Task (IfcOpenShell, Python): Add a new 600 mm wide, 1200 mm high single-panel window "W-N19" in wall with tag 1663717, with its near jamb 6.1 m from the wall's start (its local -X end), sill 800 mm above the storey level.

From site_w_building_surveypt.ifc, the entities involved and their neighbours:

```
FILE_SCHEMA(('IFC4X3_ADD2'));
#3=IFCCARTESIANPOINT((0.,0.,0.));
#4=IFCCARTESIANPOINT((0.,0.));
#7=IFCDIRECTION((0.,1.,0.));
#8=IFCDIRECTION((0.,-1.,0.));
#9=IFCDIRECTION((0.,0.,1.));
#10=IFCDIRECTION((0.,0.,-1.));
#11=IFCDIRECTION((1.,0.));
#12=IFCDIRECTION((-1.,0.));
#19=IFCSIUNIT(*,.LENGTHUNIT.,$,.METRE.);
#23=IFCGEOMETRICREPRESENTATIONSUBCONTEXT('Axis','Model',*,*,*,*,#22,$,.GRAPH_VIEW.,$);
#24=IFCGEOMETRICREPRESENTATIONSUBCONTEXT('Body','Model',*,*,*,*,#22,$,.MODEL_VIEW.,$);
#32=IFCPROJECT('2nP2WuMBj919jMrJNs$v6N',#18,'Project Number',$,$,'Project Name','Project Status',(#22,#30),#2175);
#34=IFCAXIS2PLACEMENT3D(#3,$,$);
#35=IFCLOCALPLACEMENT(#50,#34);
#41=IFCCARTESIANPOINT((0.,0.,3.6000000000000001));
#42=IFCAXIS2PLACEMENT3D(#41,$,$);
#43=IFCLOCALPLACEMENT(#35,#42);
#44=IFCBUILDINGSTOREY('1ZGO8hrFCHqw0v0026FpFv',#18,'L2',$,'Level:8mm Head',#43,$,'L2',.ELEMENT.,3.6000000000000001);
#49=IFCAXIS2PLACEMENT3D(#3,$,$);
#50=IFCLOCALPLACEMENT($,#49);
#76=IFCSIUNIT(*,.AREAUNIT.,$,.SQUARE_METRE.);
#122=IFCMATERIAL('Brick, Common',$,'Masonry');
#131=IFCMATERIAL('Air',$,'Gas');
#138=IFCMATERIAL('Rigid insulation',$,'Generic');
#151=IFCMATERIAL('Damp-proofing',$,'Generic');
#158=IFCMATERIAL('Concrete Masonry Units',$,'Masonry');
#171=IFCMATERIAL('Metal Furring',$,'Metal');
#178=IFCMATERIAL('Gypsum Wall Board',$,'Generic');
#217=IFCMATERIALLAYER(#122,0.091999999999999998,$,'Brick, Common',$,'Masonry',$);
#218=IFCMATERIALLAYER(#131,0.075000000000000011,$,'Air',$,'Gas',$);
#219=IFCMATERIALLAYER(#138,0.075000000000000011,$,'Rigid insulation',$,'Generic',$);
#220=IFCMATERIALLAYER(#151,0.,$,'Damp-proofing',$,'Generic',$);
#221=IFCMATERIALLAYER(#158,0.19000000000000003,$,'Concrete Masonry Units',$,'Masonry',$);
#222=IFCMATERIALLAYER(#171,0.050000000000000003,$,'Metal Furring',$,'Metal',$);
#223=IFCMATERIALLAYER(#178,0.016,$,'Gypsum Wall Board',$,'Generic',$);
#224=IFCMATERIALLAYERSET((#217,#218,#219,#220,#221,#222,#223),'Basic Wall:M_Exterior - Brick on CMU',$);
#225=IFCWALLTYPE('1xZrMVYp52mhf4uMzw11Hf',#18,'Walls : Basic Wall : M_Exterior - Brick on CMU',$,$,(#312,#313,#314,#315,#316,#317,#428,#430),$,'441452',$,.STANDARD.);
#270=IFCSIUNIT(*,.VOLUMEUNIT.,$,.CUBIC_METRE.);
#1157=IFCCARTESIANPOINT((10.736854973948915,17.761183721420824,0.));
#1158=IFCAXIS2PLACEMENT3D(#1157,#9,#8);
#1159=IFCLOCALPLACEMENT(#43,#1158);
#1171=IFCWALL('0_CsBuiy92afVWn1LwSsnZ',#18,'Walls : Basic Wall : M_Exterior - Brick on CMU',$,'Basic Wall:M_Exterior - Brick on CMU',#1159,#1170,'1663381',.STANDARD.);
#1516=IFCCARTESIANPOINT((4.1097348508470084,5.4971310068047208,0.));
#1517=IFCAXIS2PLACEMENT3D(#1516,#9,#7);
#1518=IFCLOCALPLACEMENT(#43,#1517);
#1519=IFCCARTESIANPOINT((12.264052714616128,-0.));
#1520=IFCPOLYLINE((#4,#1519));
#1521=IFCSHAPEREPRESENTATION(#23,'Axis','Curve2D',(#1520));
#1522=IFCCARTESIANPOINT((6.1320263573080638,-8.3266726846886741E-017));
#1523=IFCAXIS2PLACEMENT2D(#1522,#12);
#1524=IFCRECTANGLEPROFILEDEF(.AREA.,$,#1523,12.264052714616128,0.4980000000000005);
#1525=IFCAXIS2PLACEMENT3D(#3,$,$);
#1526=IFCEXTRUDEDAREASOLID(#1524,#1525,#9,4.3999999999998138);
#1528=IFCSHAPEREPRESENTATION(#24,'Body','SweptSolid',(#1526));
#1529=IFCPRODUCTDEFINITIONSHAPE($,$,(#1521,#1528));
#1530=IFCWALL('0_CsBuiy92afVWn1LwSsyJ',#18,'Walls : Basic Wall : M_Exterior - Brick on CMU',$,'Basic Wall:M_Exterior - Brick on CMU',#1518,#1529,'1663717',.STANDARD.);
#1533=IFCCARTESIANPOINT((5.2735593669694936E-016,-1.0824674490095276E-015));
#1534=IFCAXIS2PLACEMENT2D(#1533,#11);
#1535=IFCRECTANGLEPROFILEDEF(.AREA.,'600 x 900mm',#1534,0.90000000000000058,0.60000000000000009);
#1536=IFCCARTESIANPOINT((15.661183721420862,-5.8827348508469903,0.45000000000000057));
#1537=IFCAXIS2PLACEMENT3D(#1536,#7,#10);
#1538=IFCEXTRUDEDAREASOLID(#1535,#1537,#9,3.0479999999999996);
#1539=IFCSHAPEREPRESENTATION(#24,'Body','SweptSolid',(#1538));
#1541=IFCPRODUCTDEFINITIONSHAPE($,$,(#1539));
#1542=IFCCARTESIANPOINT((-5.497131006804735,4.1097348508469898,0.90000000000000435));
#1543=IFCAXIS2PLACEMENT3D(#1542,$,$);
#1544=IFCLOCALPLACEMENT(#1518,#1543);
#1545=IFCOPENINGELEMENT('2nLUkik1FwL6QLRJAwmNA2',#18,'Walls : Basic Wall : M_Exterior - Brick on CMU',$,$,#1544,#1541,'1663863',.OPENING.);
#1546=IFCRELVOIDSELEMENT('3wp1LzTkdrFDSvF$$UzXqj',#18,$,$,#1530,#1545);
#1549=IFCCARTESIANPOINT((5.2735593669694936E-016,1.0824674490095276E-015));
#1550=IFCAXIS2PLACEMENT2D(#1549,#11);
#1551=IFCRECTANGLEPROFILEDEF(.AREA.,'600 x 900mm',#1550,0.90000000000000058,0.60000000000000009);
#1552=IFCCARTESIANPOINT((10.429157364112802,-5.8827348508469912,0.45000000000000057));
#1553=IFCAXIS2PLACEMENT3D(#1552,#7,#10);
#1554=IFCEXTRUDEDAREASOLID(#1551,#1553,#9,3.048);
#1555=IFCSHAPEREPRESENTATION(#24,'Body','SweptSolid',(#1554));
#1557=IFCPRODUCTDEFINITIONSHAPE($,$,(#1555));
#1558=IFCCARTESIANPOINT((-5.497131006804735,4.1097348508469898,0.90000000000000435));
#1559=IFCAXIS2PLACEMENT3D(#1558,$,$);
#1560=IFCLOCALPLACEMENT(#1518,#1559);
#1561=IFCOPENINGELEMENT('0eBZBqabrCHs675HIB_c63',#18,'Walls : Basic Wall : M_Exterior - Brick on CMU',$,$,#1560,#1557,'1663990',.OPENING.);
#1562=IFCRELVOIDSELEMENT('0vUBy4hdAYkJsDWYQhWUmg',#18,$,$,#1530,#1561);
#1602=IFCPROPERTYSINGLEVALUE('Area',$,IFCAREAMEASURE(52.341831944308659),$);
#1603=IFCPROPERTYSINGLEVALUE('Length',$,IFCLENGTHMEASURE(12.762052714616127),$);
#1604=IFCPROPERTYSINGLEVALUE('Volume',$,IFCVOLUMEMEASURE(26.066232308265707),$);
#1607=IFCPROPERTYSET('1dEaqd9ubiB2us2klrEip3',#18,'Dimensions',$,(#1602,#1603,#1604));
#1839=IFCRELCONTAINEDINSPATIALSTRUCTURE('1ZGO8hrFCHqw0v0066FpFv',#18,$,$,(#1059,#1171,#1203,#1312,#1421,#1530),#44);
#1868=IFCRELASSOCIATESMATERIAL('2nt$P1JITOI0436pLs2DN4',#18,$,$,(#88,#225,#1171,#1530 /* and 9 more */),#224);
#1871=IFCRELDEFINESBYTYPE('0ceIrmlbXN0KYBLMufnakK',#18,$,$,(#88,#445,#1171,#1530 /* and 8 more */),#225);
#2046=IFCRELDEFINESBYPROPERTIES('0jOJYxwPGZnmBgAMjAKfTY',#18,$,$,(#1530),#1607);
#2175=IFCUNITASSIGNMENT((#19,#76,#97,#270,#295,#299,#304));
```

```python
import numpy as np
import ifcopenshell
import ifcopenshell.api.feature
import ifcopenshell.api.geometry
import ifcopenshell.api.pset
import ifcopenshell.api.root
import ifcopenshell.api.spatial
import ifcopenshell.geom
import ifcopenshell.util.element
import ifcopenshell.util.placement
import ifcopenshell.util.representation
import ifcopenshell.util.shape
import ifcopenshell.util.unit

model = ifcopenshell.open("site_w_building_surveypt.ifc")
unit_scale = ifcopenshell.util.unit.calculate_unit_scale(model)
area_scale = ifcopenshell.util.unit.calculate_unit_scale(model, "AREAUNIT")
volume_scale = ifcopenshell.util.unit.calculate_unit_scale(model, "VOLUMEUNIT")
settings = ifcopenshell.geom.settings()


def volume(element):
    """Net volume in cubic metres, openings subtracted."""
    shape = ifcopenshell.geom.create_shape(settings, element)
    return ifcopenshell.util.shape.get_volume(shape.geometry)


wall = model.by_id(1530)
storey = ifcopenshell.util.element.get_container(wall, ifc_class="IfcBuildingStorey")
context = ifcopenshell.util.representation.get_context(model, "Model", "Body", "MODEL_VIEW")
before = volume(wall)

width, height, from_end, sill = 0.6, 1.2, 6.1, 0.8  # metres

# The wall runs along its own X axis, and the end named is its -X end.
wall_shape = ifcopenshell.geom.create_shape(settings, wall)
x, y, z = ifcopenshell.util.shape.get_vertices(wall_shape.geometry).T
start = x.min() + from_end
face, thickness = float(y.min()), float(y.max() - y.min())
wall_matrix = ifcopenshell.util.placement.get_local_placement(wall.ObjectPlacement)
level = ifcopenshell.util.placement.get_local_placement(storey.ObjectPlacement)[2, 3]


def in_wall(x, y):
    """Placement at x, y metres in the wall's axes, at sill height."""
    matrix = wall_matrix.copy()
    matrix[:, 3] = wall_matrix @ np.array([x / unit_scale, y / unit_scale, 0.0, 1.0])
    matrix[2, 3] = level + sill / unit_scale
    return matrix


# Opening: a box that overshoots both wall faces by 50 mm.
opening = ifcopenshell.api.root.create_entity(model, ifc_class="IfcOpeningElement", predefined_type="OPENING")
box = ifcopenshell.api.geometry.add_wall_representation(
    model, context=context, length=width, height=height, thickness=thickness + 0.1
)
ifcopenshell.api.geometry.assign_representation(model, product=opening, representation=box)
ifcopenshell.api.geometry.edit_object_placement(model, product=opening, matrix=in_wall(start, face - 0.05), is_si=False)
ifcopenshell.api.feature.add_feature(model, feature=opening, element=wall)

window = ifcopenshell.api.root.create_entity(model, ifc_class="IfcWindow", name="W-N19", predefined_type="WINDOW")
window.OverallWidth, window.OverallHeight = width / unit_scale, height / unit_scale
window.PartitioningType = "SINGLE_PANEL"
body = ifcopenshell.api.geometry.add_window_representation(
    model,
    context=context,
    overall_width=window.OverallWidth,
    overall_height=window.OverallHeight,
    partition_type="SINGLE_PANEL",
)
ifcopenshell.api.geometry.assign_representation(model, product=window, representation=body)
ifcopenshell.api.spatial.assign_container(model, products=[window], relating_structure=storey)
ifcopenshell.api.feature.add_filling(model, opening=opening, element=window)

# Centre the window in the wall's thickness.
ifcopenshell.api.geometry.edit_object_placement(model, product=window, matrix=in_wall(start, face), is_si=False)
window_shape = ifcopenshell.geom.create_shape(settings, window)
depth = ifcopenshell.util.shape.get_vertices(window_shape.geometry)[:, 1]
offset = face + thickness / 2 - (depth.min() + depth.max()) / 2
ifcopenshell.api.geometry.edit_object_placement(model, product=window, matrix=in_wall(start, offset), is_si=False)

after = volume(wall)

# Update the wall's stored quantities.
pset = model.by_id(ifcopenshell.util.element.get_pset(wall, "Dimensions", should_inherit=False)["id"])
ifcopenshell.api.pset.edit_pset(model, pset=pset, properties={
    "Area": model.create_entity("IfcAreaMeasure", after / thickness / area_scale),
    "Volume": model.create_entity("IfcVolumeMeasure", after / volume_scale),
})

print(f"wall volume {before:.3f} -> {after:.3f} m3")

model.write("site_w_building_surveypt_updated.ifc")
```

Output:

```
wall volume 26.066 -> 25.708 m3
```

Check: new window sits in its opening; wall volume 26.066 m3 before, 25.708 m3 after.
